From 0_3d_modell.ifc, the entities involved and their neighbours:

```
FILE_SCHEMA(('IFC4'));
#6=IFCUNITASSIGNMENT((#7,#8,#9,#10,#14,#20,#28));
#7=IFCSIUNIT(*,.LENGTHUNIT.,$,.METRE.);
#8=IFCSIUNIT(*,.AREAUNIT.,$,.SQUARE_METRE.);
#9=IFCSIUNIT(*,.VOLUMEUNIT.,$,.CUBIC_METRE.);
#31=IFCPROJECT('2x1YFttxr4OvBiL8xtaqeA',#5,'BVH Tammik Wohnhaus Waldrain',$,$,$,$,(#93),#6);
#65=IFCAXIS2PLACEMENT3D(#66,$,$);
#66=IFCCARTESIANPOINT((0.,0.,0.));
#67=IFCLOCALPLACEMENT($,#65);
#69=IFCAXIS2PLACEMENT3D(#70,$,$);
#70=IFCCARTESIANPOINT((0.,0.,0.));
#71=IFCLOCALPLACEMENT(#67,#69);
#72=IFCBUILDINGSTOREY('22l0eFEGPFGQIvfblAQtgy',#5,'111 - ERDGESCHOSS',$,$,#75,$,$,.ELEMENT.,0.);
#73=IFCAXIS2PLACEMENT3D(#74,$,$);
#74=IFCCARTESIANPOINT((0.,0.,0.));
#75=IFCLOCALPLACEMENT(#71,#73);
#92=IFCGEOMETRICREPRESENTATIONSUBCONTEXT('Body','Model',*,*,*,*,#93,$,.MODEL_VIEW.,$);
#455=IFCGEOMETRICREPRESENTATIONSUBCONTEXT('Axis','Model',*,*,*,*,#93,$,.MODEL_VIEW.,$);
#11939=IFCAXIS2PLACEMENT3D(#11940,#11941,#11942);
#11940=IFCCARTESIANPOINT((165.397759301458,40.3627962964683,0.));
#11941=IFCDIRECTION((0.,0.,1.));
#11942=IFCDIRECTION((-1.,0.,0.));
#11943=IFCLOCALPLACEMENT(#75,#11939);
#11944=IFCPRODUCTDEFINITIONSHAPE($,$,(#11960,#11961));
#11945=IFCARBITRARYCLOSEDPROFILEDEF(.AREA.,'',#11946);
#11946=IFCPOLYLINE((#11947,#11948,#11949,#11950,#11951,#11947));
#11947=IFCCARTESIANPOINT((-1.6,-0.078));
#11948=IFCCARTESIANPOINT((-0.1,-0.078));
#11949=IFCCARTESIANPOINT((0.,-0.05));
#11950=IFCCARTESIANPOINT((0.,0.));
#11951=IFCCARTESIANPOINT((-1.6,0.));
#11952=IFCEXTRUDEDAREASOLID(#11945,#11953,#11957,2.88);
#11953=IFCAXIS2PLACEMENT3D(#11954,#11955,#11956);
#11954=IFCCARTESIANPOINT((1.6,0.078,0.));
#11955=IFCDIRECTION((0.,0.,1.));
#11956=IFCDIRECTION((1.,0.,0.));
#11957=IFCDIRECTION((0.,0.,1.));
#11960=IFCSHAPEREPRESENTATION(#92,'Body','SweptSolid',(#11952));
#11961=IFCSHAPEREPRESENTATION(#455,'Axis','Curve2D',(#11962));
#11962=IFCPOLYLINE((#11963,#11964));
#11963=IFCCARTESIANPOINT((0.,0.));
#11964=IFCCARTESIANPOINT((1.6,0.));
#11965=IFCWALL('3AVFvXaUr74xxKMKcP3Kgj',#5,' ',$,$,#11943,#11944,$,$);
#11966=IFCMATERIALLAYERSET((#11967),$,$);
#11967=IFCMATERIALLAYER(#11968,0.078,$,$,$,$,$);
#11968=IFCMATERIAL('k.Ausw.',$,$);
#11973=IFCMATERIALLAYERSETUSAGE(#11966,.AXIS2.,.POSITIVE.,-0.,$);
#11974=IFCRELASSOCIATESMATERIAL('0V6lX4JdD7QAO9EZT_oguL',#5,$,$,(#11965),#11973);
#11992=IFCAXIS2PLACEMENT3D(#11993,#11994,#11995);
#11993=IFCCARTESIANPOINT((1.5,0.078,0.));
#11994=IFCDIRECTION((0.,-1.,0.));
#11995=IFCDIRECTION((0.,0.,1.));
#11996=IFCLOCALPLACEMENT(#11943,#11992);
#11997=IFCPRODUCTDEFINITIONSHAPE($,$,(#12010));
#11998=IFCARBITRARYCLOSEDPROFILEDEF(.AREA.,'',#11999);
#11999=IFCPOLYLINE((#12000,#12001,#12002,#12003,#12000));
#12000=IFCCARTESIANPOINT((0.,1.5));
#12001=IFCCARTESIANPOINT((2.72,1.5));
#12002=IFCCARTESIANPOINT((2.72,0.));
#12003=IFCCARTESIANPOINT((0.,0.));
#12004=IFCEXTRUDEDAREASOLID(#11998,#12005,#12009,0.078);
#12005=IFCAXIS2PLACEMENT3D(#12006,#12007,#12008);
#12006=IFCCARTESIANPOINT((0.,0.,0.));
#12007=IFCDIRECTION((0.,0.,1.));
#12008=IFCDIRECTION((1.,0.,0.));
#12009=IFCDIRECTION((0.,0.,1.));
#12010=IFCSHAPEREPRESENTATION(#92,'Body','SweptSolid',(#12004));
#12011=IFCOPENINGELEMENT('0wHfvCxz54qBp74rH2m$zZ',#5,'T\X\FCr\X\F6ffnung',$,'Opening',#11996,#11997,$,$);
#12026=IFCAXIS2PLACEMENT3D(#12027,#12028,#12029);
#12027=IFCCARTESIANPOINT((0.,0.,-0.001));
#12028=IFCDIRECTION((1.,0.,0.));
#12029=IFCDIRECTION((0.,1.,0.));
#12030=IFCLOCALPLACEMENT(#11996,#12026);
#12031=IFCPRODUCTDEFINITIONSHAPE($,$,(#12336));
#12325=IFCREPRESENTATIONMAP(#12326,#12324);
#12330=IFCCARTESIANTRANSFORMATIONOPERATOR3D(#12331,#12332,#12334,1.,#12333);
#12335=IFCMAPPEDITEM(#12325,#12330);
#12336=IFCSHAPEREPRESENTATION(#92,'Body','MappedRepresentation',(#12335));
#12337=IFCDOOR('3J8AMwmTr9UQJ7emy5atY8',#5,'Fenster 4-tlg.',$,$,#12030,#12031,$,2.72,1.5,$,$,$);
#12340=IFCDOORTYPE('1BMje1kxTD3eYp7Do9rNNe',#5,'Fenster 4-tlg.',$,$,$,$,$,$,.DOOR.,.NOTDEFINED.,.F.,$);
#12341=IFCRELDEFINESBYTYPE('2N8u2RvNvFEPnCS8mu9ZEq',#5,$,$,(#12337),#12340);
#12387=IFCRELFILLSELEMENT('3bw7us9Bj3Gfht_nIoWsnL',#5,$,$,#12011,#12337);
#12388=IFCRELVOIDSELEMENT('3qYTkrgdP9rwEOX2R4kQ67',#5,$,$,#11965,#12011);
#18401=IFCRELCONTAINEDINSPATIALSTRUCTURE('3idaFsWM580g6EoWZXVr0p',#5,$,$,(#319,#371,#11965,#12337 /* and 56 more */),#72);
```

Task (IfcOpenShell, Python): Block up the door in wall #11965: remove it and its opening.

```python
import ifcopenshell
import ifcopenshell.api.feature
import ifcopenshell.api.root
import ifcopenshell.geom
import ifcopenshell.util.shape

model = ifcopenshell.open("0_3d_modell.ifc")
settings = ifcopenshell.geom.settings()


def volume(element):
    """Net volume in cubic metres, openings subtracted."""
    shape = ifcopenshell.geom.create_shape(settings, element)
    return ifcopenshell.util.shape.get_volume(shape.geometry)


door = model.by_guid("3J8AMwmTr9UQJ7emy5atY8")
opening = door.FillsVoids[0].RelatingOpeningElement
wall = opening.VoidsElements[0].RelatingBuildingElement
before = volume(wall)

ifcopenshell.api.root.remove_product(model, product=door)
ifcopenshell.api.feature.remove_feature(model, feature=opening)

after = volume(wall)

print(f"wall volume {before:.3f} -> {after:.3f} m3")

model.write("0_3d_modell_edited.ifc")
```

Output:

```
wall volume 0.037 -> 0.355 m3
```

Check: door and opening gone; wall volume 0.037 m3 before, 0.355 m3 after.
